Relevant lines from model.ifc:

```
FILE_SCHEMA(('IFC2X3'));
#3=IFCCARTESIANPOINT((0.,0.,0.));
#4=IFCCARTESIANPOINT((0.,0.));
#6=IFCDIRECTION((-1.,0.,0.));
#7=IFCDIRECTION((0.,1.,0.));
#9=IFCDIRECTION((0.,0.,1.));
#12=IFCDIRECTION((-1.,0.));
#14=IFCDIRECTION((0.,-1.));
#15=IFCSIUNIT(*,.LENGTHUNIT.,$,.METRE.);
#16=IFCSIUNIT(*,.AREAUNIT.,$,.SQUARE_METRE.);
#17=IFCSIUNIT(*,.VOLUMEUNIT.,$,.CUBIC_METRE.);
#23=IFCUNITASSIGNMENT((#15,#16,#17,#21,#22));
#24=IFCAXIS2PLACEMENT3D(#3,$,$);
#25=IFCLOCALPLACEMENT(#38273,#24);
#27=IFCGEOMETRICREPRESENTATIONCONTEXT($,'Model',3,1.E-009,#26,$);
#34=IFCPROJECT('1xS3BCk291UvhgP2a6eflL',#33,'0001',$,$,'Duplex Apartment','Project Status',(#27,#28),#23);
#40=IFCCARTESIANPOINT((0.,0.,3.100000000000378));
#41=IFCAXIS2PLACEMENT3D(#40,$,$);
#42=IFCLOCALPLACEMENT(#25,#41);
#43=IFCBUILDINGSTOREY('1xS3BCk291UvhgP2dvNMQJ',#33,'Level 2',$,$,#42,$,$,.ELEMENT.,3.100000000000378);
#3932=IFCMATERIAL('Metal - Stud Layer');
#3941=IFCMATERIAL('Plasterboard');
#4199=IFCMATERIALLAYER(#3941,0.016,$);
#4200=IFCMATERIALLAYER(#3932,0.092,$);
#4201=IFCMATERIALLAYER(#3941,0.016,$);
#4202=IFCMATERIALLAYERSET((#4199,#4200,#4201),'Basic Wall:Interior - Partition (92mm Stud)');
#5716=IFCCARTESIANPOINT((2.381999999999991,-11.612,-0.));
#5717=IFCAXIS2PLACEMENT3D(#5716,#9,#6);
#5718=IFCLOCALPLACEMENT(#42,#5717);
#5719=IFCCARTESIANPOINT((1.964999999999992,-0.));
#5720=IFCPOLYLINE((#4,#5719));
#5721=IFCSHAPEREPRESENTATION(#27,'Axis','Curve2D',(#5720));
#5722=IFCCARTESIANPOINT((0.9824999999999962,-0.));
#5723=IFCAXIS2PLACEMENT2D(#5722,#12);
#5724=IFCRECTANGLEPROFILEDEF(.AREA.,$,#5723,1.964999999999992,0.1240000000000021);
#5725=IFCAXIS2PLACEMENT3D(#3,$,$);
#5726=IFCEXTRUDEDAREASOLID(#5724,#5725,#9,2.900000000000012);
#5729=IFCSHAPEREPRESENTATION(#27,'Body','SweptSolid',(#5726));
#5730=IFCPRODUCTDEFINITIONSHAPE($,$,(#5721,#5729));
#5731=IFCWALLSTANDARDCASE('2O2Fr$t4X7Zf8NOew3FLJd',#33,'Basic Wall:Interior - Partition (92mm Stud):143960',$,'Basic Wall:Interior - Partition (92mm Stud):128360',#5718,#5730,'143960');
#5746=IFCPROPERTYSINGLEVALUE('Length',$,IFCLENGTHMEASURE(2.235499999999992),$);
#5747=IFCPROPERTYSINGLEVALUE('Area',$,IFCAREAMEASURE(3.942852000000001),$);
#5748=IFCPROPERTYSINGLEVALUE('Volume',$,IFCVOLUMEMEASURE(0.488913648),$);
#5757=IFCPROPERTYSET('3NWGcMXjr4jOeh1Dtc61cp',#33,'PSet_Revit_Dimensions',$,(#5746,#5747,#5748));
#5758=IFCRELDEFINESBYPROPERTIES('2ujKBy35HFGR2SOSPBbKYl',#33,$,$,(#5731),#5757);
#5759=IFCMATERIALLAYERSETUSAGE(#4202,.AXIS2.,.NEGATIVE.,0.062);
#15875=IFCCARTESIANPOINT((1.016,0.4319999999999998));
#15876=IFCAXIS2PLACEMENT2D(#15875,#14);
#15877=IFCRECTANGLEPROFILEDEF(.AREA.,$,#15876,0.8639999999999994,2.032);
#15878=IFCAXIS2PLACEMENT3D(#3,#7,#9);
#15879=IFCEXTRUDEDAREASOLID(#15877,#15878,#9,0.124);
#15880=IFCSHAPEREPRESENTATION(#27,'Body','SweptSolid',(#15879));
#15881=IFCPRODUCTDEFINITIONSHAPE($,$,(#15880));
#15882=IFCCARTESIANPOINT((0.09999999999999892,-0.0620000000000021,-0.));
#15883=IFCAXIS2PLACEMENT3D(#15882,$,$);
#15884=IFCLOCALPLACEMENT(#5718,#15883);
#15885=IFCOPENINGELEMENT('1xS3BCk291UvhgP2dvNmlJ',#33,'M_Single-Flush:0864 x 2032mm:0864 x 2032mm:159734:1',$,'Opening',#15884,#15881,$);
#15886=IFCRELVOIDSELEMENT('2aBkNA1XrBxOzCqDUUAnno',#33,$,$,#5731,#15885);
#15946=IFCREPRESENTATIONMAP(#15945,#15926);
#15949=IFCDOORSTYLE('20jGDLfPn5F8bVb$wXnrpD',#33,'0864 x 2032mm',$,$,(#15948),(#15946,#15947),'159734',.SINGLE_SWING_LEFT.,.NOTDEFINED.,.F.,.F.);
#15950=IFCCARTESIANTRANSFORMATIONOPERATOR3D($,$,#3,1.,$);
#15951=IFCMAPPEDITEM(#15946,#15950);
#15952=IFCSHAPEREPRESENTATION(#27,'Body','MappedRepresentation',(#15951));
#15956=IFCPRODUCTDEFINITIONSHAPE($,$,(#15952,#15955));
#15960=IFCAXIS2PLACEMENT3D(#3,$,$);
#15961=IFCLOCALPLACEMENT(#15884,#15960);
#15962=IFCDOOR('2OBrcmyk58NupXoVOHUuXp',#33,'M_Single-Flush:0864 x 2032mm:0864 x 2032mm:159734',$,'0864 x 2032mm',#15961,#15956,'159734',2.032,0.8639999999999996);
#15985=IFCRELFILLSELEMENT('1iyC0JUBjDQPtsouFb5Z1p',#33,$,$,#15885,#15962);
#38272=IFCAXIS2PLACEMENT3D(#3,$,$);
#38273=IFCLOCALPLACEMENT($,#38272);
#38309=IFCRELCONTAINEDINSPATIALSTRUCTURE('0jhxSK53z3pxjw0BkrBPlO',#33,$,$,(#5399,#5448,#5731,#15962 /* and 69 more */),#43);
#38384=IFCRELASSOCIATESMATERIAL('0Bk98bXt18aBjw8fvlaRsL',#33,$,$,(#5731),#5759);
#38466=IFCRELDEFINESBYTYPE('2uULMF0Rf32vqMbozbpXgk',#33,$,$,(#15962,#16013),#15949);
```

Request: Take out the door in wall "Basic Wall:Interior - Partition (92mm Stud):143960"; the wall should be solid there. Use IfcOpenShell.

```python
import ifcopenshell
import ifcopenshell.api.feature
import ifcopenshell.api.pset
import ifcopenshell.api.root
import ifcopenshell.geom
import ifcopenshell.util.element
import ifcopenshell.util.shape
import ifcopenshell.util.unit

model = ifcopenshell.open("model.ifc")
area_scale = ifcopenshell.util.unit.calculate_unit_scale(model, "AREAUNIT")
volume_scale = ifcopenshell.util.unit.calculate_unit_scale(model, "VOLUMEUNIT")
settings = ifcopenshell.geom.settings()


def volume(element):
    """Net volume in cubic metres, openings subtracted."""
    shape = ifcopenshell.geom.create_shape(settings, element)
    return ifcopenshell.util.shape.get_volume(shape.geometry)


door = model.by_id(15962)
opening = door.FillsVoids[0].RelatingOpeningElement
wall = opening.VoidsElements[0].RelatingBuildingElement
before = volume(wall)

ifcopenshell.api.root.remove_product(model, product=door)
ifcopenshell.api.feature.remove_feature(model, feature=opening)

after = volume(wall)
thickness = 0.124  # wall thickness in metres

# Update the wall's stored quantities.
pset = model.by_id(ifcopenshell.util.element.get_pset(wall, "PSet_Revit_Dimensions", should_inherit=False)["id"])
ifcopenshell.api.pset.edit_pset(model, pset=pset, properties={
    "Area": model.create_entity("IfcAreaMeasure", after / thickness / area_scale),
    "Volume": model.create_entity("IfcVolumeMeasure", after / volume_scale),
})

print(f"wall volume {before:.3f} -> {after:.3f} m3")

model.write("model_v2.ifc")
```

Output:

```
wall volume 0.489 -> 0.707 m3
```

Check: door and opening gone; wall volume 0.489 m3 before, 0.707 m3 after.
